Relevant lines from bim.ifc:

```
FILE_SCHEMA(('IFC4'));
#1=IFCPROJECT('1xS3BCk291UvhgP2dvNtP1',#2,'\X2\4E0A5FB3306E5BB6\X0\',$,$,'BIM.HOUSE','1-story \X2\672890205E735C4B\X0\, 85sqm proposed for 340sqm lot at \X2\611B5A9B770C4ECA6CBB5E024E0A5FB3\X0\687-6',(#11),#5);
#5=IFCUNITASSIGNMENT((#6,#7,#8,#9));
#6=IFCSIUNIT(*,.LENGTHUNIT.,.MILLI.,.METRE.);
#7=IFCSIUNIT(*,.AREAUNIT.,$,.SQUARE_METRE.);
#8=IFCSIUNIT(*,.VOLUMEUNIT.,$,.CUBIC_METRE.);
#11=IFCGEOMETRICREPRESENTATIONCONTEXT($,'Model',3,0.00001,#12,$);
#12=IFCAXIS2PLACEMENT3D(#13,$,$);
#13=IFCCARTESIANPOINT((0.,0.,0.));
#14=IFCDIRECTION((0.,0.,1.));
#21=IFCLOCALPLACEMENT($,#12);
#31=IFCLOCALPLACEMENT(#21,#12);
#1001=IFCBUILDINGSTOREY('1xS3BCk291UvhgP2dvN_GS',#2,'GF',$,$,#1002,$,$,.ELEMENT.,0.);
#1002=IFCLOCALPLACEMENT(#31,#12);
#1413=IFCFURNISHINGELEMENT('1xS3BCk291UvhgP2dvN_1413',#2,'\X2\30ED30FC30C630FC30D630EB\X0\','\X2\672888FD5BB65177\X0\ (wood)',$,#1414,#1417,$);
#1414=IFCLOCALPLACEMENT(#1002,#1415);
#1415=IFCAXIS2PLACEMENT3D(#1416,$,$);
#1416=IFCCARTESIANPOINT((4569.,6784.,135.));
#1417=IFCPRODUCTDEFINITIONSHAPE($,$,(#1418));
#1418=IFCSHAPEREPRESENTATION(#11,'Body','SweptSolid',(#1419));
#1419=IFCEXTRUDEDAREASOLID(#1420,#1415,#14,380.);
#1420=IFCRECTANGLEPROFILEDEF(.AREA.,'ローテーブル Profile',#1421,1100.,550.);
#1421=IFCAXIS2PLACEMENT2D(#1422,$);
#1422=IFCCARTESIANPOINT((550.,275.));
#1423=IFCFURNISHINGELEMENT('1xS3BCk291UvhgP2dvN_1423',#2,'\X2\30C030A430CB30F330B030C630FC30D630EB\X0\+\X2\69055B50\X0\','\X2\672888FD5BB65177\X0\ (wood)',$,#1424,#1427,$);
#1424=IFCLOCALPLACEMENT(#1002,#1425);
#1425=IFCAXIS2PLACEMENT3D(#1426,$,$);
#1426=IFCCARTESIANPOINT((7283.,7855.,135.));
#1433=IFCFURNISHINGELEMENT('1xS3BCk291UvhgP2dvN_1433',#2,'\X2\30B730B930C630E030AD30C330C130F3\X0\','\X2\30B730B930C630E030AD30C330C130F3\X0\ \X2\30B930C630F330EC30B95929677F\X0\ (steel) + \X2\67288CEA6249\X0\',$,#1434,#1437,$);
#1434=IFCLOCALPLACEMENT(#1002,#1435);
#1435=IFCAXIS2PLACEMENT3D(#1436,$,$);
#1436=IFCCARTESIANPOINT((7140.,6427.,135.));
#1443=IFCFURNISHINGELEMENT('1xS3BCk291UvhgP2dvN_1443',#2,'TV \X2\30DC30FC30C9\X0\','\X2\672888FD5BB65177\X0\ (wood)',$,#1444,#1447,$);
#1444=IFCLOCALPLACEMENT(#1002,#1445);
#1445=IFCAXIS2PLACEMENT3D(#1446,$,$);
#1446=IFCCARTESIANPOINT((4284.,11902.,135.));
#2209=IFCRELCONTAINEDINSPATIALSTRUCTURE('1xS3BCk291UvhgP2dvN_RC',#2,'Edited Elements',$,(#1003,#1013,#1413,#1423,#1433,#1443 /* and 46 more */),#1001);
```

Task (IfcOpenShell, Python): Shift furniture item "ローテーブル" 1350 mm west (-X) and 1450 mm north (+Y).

```python
import ifcopenshell
import ifcopenshell.api.geometry
import ifcopenshell.util.placement

model = ifcopenshell.open("bim.ifc")

item = model.by_guid("1xS3BCk291UvhgP2dvN_1413")
matrix = ifcopenshell.util.placement.get_local_placement(item.ObjectPlacement)
matrix[0, 3] -= 1350.0
matrix[1, 3] += 1450.0
ifcopenshell.api.geometry.edit_object_placement(model, product=item, matrix=matrix, is_si=False)

print(ifcopenshell.util.placement.get_local_placement(item.ObjectPlacement).round(3) + 0.0)

model.write("bim_rev.ifc")
```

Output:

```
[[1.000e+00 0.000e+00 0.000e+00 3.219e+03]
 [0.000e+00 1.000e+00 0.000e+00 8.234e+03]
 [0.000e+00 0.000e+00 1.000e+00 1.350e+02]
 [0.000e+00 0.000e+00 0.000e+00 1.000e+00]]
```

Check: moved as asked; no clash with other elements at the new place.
